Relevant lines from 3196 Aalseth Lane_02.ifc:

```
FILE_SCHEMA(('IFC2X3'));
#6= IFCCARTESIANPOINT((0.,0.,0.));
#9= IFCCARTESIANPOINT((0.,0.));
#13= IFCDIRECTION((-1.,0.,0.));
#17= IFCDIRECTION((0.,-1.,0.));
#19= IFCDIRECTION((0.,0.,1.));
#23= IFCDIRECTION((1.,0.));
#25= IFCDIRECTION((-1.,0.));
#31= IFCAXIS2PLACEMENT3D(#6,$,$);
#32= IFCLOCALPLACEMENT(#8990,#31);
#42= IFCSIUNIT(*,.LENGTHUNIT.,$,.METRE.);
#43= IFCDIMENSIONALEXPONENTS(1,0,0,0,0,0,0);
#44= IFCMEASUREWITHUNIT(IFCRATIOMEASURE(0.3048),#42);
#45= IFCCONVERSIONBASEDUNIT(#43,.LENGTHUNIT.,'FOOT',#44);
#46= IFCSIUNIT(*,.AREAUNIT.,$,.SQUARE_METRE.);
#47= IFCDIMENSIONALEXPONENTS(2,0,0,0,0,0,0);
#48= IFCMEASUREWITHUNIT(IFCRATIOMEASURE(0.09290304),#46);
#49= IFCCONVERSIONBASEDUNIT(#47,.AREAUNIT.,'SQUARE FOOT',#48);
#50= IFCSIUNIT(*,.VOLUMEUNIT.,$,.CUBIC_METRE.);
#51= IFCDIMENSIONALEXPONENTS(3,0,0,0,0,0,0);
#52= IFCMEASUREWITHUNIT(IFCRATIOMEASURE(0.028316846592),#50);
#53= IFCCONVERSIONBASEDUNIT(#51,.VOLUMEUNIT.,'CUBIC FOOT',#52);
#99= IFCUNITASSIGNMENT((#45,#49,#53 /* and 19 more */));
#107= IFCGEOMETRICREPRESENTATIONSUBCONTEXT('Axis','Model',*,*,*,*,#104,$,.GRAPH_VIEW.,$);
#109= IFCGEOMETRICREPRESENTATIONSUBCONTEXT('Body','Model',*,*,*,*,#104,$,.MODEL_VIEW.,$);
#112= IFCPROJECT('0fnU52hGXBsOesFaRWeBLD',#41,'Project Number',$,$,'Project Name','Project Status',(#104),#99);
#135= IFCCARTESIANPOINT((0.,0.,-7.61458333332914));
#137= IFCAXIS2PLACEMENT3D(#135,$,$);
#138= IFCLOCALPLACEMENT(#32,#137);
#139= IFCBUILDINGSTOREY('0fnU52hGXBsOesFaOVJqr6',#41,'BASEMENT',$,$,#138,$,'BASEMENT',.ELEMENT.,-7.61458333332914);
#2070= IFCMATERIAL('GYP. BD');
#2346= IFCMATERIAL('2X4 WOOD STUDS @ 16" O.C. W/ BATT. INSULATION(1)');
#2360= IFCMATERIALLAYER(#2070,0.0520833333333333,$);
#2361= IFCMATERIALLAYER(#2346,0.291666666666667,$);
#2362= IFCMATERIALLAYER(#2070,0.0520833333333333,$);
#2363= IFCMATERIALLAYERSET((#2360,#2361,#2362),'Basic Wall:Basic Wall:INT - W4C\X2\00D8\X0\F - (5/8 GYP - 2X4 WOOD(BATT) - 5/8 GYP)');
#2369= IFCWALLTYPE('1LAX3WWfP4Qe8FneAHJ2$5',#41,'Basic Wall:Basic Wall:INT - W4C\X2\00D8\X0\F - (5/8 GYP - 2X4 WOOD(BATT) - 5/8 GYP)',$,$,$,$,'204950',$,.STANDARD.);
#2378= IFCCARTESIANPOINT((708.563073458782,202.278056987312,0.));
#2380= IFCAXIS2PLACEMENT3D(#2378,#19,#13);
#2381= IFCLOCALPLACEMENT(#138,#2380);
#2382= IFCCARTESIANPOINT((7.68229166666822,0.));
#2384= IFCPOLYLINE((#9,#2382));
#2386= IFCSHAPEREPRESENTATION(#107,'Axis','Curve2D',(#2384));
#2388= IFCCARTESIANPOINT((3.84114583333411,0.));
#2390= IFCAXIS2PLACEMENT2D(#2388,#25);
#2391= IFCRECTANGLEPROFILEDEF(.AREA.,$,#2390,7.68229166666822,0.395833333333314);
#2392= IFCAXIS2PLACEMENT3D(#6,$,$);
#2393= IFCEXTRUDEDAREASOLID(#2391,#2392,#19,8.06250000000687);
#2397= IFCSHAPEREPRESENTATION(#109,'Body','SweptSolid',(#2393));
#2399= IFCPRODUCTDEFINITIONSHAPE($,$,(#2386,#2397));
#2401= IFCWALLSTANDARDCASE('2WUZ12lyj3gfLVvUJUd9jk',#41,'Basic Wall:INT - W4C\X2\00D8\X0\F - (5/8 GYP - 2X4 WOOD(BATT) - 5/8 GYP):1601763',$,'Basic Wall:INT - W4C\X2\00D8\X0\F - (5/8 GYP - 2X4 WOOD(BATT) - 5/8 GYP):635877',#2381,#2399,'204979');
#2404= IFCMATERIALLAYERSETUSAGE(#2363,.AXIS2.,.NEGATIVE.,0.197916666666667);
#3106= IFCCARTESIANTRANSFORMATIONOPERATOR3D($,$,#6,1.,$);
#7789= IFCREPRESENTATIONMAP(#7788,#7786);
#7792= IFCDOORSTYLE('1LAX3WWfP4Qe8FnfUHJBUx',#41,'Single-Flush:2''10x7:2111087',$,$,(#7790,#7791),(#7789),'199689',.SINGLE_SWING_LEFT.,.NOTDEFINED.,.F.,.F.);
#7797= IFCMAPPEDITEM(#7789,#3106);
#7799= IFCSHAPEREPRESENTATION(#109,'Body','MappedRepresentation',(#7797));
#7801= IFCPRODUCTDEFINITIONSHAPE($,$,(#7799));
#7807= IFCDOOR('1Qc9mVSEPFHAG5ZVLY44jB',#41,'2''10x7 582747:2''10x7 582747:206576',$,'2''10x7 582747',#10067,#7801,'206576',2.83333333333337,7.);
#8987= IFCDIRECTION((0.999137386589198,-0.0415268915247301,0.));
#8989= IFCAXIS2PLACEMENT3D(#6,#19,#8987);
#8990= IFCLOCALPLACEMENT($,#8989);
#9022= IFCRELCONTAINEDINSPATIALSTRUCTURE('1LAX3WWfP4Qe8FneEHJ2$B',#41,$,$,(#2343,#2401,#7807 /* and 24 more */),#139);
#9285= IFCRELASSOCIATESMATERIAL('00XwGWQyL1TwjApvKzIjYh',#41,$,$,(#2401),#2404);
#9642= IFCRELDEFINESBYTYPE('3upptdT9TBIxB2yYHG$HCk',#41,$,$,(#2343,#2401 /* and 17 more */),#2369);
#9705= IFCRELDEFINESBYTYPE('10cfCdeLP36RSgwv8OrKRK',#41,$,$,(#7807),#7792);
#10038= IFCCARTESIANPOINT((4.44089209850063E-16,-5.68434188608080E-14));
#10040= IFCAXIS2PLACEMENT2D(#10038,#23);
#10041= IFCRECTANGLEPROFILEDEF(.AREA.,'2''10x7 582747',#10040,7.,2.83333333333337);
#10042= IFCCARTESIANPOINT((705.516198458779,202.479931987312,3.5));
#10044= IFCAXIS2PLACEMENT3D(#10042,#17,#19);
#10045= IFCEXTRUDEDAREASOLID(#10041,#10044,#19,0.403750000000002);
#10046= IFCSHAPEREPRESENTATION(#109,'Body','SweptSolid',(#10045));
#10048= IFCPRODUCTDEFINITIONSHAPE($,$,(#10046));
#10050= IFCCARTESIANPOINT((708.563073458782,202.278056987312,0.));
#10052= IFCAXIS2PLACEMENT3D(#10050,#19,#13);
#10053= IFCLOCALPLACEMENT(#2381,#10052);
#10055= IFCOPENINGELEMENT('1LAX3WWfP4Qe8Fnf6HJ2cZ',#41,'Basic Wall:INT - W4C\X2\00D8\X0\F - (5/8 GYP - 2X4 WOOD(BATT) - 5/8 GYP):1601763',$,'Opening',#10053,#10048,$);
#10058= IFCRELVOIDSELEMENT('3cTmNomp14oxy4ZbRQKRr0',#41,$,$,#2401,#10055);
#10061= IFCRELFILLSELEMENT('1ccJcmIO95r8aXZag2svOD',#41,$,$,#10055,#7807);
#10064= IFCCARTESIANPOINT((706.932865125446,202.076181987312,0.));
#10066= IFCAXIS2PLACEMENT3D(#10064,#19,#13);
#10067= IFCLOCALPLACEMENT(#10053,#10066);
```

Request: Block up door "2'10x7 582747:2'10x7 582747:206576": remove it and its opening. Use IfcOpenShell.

```python
import ifcopenshell
import ifcopenshell.api.feature
import ifcopenshell.api.root
import ifcopenshell.geom
import ifcopenshell.util.shape

model = ifcopenshell.open("3196 Aalseth Lane_02.ifc")
settings = ifcopenshell.geom.settings()


def volume(element):
    """Net volume in cubic metres, openings subtracted."""
    shape = ifcopenshell.geom.create_shape(settings, element)
    return ifcopenshell.util.shape.get_volume(shape.geometry)


door = model.by_id(7807)
opening = door.FillsVoids[0].RelatingOpeningElement
wall = opening.VoidsElements[0].RelatingBuildingElement
before = volume(wall)

ifcopenshell.api.root.remove_product(model, product=door)
ifcopenshell.api.feature.remove_feature(model, feature=opening)

after = volume(wall)

print(f"wall volume {before:.3f} -> {after:.3f} m3")

model.write("3196 Aalseth Lane_02-out.ifc")
```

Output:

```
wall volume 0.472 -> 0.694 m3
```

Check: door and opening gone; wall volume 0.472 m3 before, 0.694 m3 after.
